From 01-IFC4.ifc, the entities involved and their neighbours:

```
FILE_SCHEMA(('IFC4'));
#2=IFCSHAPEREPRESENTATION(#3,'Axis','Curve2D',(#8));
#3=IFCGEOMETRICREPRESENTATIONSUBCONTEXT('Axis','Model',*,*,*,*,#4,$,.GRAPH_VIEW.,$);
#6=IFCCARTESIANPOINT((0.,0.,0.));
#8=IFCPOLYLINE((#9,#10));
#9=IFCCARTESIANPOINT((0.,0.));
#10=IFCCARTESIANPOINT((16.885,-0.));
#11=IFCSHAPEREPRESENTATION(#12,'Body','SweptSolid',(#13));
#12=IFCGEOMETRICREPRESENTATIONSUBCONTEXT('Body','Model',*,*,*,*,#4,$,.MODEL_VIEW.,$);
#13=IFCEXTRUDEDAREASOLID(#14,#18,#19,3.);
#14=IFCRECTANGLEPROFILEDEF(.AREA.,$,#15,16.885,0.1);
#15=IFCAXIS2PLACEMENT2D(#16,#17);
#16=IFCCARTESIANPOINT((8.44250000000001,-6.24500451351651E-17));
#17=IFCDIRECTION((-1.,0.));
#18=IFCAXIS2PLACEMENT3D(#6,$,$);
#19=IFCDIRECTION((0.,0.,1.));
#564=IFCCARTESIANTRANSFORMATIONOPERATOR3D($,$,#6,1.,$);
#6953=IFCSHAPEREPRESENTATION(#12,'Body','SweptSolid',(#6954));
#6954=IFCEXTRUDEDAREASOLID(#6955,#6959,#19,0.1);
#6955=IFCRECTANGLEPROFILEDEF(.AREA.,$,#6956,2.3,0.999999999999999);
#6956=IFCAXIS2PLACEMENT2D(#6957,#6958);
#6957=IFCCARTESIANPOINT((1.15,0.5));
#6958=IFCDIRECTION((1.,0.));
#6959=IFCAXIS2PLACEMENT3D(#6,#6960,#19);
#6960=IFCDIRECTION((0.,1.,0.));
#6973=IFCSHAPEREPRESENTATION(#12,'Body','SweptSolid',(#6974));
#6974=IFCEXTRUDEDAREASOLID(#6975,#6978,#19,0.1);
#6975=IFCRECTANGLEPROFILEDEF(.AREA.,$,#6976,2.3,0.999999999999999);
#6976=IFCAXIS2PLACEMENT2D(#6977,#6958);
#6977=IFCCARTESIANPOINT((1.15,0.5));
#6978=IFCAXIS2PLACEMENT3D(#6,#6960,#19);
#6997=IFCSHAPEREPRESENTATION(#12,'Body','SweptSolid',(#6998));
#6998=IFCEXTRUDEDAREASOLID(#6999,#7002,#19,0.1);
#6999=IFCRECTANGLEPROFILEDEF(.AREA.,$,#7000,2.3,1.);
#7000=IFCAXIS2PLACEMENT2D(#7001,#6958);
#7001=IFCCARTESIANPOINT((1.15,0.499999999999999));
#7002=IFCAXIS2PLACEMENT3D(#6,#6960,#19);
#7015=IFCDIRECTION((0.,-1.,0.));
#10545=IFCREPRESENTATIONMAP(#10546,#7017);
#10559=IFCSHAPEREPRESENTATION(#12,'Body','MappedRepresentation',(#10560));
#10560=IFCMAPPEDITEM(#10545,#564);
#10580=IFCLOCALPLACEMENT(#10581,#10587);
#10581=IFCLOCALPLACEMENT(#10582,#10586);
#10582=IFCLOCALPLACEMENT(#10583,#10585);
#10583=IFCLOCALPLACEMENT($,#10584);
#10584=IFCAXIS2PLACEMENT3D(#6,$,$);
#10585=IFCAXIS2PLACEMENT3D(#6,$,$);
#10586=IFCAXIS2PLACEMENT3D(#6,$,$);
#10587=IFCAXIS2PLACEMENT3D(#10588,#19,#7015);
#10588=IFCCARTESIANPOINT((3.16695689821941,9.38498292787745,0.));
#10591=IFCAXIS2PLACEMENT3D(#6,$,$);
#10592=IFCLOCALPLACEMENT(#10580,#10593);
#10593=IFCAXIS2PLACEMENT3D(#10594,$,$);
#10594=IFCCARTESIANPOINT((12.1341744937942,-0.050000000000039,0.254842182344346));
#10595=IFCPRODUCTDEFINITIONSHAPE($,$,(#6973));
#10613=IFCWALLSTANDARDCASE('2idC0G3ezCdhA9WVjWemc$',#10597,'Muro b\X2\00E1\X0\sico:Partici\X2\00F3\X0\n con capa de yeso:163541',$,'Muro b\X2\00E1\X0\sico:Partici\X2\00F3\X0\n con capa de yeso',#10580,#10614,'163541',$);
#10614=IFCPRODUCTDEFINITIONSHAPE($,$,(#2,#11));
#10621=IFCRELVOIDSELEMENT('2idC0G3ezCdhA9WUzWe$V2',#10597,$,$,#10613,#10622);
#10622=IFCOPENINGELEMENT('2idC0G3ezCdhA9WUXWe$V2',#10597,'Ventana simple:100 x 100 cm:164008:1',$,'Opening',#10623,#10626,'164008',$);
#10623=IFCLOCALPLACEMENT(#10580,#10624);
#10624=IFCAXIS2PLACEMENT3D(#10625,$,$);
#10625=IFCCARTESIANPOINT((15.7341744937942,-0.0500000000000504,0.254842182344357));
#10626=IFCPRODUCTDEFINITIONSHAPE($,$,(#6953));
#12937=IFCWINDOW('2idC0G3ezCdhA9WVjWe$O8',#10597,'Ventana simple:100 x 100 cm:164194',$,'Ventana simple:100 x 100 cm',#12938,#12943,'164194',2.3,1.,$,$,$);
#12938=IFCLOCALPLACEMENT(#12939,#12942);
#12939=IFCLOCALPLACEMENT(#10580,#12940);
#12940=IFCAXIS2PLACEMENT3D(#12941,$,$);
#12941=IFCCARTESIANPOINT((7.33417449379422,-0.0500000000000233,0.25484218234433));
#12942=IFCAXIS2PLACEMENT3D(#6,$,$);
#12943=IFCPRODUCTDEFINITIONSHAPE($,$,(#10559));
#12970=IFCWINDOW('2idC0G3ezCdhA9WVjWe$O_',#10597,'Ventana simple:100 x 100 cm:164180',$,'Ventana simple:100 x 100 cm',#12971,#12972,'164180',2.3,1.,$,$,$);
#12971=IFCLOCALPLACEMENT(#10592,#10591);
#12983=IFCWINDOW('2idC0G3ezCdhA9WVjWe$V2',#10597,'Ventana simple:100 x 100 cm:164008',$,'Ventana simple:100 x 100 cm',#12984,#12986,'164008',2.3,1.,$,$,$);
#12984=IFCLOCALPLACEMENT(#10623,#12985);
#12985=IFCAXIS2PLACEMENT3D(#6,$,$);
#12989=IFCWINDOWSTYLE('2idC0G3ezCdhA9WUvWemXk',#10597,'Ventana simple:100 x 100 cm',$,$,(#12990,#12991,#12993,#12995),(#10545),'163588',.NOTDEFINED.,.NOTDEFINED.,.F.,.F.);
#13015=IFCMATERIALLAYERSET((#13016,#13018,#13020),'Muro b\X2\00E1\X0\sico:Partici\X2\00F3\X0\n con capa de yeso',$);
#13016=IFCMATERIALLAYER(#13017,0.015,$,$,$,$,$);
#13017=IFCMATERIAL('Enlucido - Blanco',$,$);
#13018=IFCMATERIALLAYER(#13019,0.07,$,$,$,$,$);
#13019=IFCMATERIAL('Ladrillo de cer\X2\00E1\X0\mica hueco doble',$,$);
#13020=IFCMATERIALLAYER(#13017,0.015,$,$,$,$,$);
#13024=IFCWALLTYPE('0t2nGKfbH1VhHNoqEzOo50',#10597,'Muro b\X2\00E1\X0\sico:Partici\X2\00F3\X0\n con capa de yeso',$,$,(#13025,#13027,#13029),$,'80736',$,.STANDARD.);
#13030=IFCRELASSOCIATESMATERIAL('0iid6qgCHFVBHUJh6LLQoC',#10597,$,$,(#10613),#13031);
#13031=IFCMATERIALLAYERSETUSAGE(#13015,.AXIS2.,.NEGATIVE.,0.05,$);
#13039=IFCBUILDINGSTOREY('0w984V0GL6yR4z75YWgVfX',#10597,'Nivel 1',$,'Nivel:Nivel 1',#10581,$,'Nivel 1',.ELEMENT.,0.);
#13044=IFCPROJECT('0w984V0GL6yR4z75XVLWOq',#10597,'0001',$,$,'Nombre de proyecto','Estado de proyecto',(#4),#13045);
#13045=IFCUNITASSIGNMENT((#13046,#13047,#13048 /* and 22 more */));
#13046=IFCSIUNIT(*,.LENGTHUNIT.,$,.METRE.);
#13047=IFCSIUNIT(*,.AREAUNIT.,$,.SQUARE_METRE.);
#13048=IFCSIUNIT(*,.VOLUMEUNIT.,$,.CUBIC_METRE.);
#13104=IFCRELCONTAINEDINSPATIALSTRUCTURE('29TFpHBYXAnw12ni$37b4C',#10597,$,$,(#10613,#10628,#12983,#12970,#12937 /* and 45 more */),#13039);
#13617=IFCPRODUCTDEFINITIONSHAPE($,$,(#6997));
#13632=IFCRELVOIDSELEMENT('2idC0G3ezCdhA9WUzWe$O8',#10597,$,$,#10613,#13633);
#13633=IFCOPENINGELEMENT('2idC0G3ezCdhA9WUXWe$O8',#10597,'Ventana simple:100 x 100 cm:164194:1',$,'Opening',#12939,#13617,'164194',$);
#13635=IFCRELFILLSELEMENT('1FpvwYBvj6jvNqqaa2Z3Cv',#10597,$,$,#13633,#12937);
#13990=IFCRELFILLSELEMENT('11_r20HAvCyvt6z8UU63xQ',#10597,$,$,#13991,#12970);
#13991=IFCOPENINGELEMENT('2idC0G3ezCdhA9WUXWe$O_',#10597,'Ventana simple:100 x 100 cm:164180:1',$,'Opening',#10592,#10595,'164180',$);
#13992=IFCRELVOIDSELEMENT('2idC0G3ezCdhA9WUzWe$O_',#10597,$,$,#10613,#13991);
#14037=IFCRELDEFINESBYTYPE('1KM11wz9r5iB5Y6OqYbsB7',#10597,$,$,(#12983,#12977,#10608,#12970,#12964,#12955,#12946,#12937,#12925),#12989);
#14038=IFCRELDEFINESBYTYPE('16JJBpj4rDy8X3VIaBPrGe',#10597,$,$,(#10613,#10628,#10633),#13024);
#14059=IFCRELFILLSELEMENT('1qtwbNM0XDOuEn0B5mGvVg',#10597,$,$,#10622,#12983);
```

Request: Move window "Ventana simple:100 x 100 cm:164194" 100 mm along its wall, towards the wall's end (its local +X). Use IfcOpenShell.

```python
import ifcopenshell
import ifcopenshell.api.geometry
import ifcopenshell.util.placement

model = ifcopenshell.open("01-IFC4.ifc")

window = model.by_guid("2idC0G3ezCdhA9WVjWe$O8")
opening = window.FillsVoids[0].RelatingOpeningElement
wall = opening.VoidsElements[0].RelatingBuildingElement

wall_matrix = ifcopenshell.util.placement.get_local_placement(wall.ObjectPlacement)
shift = wall_matrix[:3, 0] * 0.1
before = ifcopenshell.util.placement.get_local_placement(window.ObjectPlacement)[:3, 3].copy()

# The window is placed relative to its opening, so it follows when the opening moves.
matrix = ifcopenshell.util.placement.get_local_placement(opening.ObjectPlacement)
matrix[:3, 3] += shift
ifcopenshell.api.geometry.edit_object_placement(
    model, product=opening, matrix=matrix, is_si=False, should_transform_children=True
)

after = ifcopenshell.util.placement.get_local_placement(window.ObjectPlacement)[:3, 3]
print("window moved by", (after - before).round(3) + 0.0)

model.write("01-IFC4-out.ifc")
```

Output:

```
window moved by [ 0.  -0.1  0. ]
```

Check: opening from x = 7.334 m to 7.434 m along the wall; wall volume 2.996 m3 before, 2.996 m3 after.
